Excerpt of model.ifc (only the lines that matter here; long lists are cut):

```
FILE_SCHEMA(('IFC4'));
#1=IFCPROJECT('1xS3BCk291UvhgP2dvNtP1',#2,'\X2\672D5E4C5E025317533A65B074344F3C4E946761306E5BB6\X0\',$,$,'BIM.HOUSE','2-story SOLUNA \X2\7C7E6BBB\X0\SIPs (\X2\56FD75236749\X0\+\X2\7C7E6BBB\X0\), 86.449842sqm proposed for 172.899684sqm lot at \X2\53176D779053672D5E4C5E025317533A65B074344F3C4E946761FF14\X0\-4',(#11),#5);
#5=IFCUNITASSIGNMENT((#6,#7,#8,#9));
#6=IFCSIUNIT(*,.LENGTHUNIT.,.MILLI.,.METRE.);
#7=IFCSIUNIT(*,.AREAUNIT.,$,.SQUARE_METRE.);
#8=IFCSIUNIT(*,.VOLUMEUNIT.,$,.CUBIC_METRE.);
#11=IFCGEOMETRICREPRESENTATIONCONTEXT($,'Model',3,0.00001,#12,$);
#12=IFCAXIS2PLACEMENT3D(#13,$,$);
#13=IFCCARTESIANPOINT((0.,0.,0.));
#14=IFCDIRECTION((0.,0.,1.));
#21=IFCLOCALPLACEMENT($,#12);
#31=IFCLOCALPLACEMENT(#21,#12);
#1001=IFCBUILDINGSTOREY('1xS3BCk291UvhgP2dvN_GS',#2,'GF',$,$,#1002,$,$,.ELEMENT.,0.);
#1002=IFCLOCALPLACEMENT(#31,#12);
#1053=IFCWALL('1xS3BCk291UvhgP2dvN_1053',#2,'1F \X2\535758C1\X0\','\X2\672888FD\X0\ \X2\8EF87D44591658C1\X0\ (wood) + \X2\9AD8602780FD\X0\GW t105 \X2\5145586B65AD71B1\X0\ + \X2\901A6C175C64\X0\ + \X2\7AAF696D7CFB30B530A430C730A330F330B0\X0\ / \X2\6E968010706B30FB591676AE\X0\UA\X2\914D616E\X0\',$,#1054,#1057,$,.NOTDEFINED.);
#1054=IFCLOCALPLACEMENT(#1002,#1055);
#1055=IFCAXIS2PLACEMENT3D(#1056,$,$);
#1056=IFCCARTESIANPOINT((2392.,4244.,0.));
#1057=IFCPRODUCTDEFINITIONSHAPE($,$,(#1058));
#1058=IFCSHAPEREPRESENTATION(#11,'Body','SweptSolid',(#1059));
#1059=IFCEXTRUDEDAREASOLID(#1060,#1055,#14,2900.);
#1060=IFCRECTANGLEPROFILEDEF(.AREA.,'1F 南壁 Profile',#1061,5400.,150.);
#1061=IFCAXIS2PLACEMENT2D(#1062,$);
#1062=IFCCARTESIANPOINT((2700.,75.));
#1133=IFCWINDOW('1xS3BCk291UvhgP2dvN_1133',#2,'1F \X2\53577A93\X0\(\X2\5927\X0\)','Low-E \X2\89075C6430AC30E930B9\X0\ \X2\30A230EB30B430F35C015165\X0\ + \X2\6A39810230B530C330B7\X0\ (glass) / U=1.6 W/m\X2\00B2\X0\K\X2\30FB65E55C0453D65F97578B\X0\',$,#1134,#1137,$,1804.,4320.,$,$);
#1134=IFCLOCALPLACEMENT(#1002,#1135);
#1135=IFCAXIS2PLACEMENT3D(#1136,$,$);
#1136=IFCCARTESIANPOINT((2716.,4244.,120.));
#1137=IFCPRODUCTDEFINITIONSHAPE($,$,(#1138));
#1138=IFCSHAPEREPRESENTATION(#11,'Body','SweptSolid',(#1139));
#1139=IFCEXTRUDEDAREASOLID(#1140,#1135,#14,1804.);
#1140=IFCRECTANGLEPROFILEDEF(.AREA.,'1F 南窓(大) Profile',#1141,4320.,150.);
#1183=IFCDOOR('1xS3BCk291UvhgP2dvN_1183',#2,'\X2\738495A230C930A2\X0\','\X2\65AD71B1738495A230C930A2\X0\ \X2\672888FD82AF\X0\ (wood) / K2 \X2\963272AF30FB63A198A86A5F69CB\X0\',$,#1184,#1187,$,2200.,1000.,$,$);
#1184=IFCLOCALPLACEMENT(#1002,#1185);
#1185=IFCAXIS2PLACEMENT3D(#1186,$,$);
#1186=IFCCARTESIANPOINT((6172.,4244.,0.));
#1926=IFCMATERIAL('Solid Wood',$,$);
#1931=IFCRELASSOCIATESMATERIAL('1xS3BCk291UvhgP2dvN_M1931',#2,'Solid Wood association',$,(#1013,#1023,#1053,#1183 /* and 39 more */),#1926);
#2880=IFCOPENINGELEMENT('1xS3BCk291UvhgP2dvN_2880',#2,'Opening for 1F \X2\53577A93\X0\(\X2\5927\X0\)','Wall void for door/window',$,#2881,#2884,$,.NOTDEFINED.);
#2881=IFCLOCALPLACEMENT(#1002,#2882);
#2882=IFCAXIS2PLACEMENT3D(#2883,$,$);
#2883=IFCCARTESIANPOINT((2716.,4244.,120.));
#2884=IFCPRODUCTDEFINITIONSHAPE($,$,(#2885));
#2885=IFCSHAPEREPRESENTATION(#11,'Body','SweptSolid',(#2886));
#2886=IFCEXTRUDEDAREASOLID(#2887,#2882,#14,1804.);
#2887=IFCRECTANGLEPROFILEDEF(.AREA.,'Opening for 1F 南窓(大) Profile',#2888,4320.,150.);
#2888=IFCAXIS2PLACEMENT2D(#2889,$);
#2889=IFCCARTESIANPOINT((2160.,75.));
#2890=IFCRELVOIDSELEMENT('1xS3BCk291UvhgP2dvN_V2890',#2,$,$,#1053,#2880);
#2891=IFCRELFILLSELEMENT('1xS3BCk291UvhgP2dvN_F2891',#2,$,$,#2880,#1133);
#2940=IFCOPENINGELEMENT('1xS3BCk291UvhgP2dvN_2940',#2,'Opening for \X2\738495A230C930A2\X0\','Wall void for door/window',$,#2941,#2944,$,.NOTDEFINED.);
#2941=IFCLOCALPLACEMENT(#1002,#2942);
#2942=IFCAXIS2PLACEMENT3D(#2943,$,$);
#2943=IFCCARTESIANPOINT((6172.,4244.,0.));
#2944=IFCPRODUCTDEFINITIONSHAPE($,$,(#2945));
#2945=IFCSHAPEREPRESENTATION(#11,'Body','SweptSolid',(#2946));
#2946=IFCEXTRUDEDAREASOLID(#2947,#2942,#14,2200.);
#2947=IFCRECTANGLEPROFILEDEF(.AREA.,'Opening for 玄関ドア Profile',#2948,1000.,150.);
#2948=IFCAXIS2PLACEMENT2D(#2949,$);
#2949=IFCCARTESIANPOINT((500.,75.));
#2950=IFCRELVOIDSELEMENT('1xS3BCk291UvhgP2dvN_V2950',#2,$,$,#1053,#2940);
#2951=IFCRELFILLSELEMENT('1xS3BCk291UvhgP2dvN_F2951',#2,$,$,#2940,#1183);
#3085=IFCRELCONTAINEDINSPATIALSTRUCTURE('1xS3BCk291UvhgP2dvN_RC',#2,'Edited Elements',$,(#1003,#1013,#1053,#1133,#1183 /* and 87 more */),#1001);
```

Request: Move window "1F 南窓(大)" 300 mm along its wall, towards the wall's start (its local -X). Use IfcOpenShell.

```python
import ifcopenshell
import ifcopenshell.api.geometry
import ifcopenshell.util.placement
import ifcopenshell.util.unit

model = ifcopenshell.open("model.ifc")
unit_scale = ifcopenshell.util.unit.calculate_unit_scale(model)

window = model.by_id(1133)
opening = window.FillsVoids[0].RelatingOpeningElement
wall = opening.VoidsElements[0].RelatingBuildingElement

wall_matrix = ifcopenshell.util.placement.get_local_placement(wall.ObjectPlacement)
shift = wall_matrix[:3, 0] * -0.3 / unit_scale
before = ifcopenshell.util.placement.get_local_placement(window.ObjectPlacement)[:3, 3].copy()

# The window is not placed relative to its opening, so move both.
for product in (opening, window):
    matrix = ifcopenshell.util.placement.get_local_placement(product.ObjectPlacement)
    matrix[:3, 3] += shift
    ifcopenshell.api.geometry.edit_object_placement(model, product=product, matrix=matrix, is_si=False)

after = ifcopenshell.util.placement.get_local_placement(window.ObjectPlacement)[:3, 3]
print("window moved by", (after - before).round(3) + 0.0)

model.write("model_edited.ifc")
```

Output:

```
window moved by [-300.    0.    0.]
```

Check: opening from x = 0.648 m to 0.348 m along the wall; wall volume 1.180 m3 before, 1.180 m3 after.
